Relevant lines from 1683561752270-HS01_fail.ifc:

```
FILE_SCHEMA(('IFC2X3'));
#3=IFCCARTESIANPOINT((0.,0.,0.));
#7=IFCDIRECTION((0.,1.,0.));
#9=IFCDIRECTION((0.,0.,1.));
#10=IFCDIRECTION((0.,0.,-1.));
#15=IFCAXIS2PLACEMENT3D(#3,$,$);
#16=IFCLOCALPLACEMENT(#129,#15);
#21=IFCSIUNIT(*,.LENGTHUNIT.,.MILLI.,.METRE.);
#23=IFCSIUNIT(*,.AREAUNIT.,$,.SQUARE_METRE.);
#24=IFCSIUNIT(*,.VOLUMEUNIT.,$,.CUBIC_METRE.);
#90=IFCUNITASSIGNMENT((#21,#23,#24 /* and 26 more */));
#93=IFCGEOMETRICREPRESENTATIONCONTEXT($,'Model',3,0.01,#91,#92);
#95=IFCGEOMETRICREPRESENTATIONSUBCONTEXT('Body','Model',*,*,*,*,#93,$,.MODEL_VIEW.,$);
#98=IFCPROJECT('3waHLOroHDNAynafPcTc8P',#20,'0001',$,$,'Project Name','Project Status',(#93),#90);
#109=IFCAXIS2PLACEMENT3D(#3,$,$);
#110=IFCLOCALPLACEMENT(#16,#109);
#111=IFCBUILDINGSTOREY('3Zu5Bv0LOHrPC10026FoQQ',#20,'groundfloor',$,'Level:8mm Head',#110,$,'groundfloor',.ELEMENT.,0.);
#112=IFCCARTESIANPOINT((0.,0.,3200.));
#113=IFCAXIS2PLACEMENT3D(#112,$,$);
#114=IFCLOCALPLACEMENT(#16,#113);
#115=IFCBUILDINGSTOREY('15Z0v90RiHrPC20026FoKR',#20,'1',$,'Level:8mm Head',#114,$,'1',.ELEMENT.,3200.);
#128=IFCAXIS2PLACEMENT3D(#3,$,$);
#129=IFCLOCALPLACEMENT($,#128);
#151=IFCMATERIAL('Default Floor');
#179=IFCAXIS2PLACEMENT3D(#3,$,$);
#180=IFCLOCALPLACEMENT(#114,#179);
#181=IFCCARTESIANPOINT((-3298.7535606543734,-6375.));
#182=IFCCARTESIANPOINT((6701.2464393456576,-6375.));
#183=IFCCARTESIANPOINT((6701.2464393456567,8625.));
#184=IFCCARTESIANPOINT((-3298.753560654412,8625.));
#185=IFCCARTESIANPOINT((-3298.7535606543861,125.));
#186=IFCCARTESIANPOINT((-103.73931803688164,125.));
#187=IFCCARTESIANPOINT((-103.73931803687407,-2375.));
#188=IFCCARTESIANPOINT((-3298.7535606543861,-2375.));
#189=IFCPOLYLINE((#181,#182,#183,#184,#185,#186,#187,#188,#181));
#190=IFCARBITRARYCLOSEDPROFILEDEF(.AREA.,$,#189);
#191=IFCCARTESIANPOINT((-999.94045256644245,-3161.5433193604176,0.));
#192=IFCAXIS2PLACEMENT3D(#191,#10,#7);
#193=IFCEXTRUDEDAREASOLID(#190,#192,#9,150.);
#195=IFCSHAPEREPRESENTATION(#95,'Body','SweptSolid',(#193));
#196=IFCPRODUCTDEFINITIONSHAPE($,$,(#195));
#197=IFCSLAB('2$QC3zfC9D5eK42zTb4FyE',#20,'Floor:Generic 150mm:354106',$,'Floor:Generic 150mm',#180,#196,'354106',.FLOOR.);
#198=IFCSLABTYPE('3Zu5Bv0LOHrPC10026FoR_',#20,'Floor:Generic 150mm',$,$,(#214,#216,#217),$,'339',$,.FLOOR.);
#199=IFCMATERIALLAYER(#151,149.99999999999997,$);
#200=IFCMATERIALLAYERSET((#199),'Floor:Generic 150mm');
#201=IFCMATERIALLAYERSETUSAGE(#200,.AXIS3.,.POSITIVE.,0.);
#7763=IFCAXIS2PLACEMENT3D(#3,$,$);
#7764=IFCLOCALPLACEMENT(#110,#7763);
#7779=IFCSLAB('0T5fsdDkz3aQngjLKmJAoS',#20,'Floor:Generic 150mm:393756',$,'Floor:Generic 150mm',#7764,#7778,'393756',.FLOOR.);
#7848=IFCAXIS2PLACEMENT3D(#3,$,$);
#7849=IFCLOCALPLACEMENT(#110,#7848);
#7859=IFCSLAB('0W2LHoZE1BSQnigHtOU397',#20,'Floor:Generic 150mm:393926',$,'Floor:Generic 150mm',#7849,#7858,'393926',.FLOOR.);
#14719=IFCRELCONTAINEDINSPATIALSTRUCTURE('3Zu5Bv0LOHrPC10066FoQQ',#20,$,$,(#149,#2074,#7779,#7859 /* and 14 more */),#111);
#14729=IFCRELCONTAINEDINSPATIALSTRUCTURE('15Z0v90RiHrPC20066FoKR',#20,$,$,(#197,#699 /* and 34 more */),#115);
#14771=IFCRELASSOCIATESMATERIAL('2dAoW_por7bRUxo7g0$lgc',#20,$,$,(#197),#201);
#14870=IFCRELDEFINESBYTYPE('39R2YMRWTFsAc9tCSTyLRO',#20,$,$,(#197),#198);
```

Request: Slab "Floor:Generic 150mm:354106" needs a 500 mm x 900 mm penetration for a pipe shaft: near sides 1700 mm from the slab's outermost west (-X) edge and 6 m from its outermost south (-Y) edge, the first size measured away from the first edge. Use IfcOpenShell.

```python
import numpy as np
import ifcopenshell
import ifcopenshell.api.feature
import ifcopenshell.api.geometry
import ifcopenshell.api.root
import ifcopenshell.geom
import ifcopenshell.util.placement
import ifcopenshell.util.representation
import ifcopenshell.util.shape
import ifcopenshell.util.unit

model = ifcopenshell.open("1683561752270-HS01_fail.ifc")
unit_scale = ifcopenshell.util.unit.calculate_unit_scale(model)
settings = ifcopenshell.geom.settings()


def volume(element):
    """Net volume in cubic metres, openings subtracted."""
    shape = ifcopenshell.geom.create_shape(settings, element)
    return ifcopenshell.util.shape.get_volume(shape.geometry)


slab = model.by_id(197)
before = volume(slab)

# Extent in the slab's own axes, in metres. The edges named are its -X and -Y sides.
slab_shape = ifcopenshell.geom.create_shape(settings, slab)
vertices = ifcopenshell.util.shape.get_vertices(slab_shape.geometry)
x_min, y_min, bottom = vertices.min(axis=0)
top = vertices[:, 2].max()

opening = ifcopenshell.api.root.create_entity(model, ifc_class="IfcOpeningElement", name="Pipe shaft opening")
context = ifcopenshell.util.representation.get_context(model, "Model", "Body", "MODEL_VIEW")
width, depth = 0.5, 0.9
outline = [(0.0, 0.0), (width, 0.0), (width, depth), (0.0, depth), (0.0, 0.0)]
# Overshoot both faces by 50 mm so the cut is clean.
shape = ifcopenshell.api.geometry.add_slab_representation(
    model, context=context, depth=top - bottom + 0.1, polyline=outline
)
ifcopenshell.api.geometry.assign_representation(model, product=opening, representation=shape)

matrix = ifcopenshell.util.placement.get_local_placement(slab.ObjectPlacement)
matrix[:, 3] = matrix @ np.append(np.array([x_min + 1.7, y_min + 6, bottom - 0.05]) / unit_scale, 1.0)
ifcopenshell.api.geometry.edit_object_placement(model, product=opening, matrix=matrix, is_si=False)
ifcopenshell.api.feature.add_feature(model, feature=opening, element=slab)

after = volume(slab)

print(f"slab volume {before:.3f} -> {after:.3f} m3")

model.write("1683561752270-HS01_fail_edited.ifc")
```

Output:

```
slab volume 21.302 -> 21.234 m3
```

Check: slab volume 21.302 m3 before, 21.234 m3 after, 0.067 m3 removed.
